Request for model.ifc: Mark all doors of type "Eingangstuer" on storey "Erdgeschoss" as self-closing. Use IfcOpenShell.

First a look at what the model holds.

```python
import ifcopenshell
import ifcopenshell.util.element

model = ifcopenshell.open("model.ifc")
print(model.schema)
storey = next(s for s in model.by_type("IfcBuildingStorey") if s.Name == "Erdgeschoss")
doors = [e for e in ifcopenshell.util.element.get_decomposition(storey) if e.is_a("IfcDoor")]
seen = {}
for e in doors:
    element_type = ifcopenshell.util.element.get_type(e)
    key = (element_type.Name if element_type != e and element_type else None, ifcopenshell.util.element.get_pset(e, "Pset_DoorCommon", "SelfClosing"))
    seen[key] = seen.get(key, 0) + 1
for (name, value), count in sorted(seen.items(), key=str):
    print(count, "x", name, "|", value)
```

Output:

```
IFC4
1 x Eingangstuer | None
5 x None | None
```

```python
import ifcopenshell
import ifcopenshell.api.pset
import ifcopenshell.util.element

model = ifcopenshell.open("model.ifc")

storey = next(s for s in model.by_type("IfcBuildingStorey") if s.Name == "Erdgeschoss")
doors = [e for e in ifcopenshell.util.element.get_decomposition(storey) if e.is_a("IfcDoor")]

count = 0
for e in doors:
    element_type = ifcopenshell.util.element.get_type(e)
    if element_type in (None, e) or element_type.Name != "Eingangstuer":
        continue
    # add_pset returns the element's existing set when there is one.
    pset = ifcopenshell.api.pset.add_pset(model, product=e, name="Pset_DoorCommon")
    ifcopenshell.api.pset.edit_pset(model, pset=pset, properties={"SelfClosing": True})
    count += 1

print(count, "doors updated")

model.write("model_edited.ifc")
```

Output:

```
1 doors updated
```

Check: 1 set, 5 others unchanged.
